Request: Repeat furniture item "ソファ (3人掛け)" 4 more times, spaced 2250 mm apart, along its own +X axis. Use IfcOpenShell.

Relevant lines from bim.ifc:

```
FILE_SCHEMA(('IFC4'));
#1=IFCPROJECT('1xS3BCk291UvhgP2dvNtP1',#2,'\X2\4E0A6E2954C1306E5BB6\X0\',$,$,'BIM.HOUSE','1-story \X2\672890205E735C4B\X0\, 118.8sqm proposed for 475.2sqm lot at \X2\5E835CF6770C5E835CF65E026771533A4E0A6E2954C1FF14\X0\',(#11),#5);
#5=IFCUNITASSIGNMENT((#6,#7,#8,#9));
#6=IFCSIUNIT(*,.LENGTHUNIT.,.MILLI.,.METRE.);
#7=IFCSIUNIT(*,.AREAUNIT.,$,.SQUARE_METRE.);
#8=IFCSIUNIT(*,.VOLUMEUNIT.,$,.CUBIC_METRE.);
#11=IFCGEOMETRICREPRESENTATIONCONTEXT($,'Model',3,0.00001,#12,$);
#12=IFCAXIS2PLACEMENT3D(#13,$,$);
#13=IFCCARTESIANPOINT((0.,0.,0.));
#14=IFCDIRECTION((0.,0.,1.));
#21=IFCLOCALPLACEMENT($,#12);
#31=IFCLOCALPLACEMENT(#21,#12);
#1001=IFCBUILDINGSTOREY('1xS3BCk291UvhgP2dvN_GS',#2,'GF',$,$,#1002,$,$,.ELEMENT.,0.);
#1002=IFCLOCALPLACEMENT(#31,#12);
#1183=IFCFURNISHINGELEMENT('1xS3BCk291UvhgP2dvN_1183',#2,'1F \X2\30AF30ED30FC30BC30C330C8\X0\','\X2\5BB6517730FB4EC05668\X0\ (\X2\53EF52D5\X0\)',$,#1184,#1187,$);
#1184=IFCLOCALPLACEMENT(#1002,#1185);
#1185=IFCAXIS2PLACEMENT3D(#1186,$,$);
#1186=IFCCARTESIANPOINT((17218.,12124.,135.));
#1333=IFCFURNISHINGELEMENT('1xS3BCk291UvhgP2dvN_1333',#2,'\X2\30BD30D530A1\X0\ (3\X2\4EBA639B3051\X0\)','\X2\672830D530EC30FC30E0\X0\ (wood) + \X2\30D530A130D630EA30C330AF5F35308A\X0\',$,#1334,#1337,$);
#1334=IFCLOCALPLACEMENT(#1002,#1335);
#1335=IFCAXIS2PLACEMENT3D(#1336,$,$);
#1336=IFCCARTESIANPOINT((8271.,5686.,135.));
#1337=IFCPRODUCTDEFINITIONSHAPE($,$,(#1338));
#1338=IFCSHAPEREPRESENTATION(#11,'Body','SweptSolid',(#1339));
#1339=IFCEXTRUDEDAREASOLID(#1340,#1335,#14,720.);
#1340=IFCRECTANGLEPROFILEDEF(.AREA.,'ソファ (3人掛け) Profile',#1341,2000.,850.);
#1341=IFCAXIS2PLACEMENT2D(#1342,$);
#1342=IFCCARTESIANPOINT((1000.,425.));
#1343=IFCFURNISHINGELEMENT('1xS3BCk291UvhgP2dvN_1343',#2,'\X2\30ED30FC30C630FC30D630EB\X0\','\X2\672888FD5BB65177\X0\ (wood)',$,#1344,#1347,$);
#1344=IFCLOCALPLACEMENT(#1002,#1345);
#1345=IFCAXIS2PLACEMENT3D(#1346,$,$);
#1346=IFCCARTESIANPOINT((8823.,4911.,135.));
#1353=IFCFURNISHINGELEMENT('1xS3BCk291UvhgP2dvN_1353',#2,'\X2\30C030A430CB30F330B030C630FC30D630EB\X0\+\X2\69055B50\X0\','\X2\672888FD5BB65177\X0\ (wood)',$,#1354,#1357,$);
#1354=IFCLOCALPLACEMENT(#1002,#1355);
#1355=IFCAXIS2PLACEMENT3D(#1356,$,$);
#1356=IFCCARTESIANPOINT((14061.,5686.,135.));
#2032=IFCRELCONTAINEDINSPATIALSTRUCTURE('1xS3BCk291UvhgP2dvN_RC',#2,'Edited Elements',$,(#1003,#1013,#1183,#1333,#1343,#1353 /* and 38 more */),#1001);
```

```python
import ifcopenshell
import ifcopenshell.api.geometry
import ifcopenshell.api.root
import ifcopenshell.util.element
import ifcopenshell.util.placement
import ifcopenshell.util.unit

model = ifcopenshell.open("bim.ifc")
unit_scale = ifcopenshell.util.unit.calculate_unit_scale(model)


def reuse_history(source, copy):
    """copy_class also copies each property set's owner history, people and application; keep the originals."""
    for rel in copy.IsDefinedBy:
        if rel.is_a("IfcRelDefinesByProperties") and (history := rel.RelatingPropertyDefinition.OwnerHistory):
            rel.RelatingPropertyDefinition.OwnerHistory = source.OwnerHistory
            ifcopenshell.util.element.remove_deep2(model, history)


source = model.by_id(1333)
base = ifcopenshell.util.placement.get_local_placement(source.ObjectPlacement)
step = base[:3, 0] * 2.25 / unit_scale

for i in range(1, 5):
    copy = ifcopenshell.api.root.copy_class(model, product=source)
    copy.Representation = ifcopenshell.util.element.copy_deep(
        model, source.Representation, exclude=["IfcGeometricRepresentationContext", "IfcRepresentationMap"]
    )
    reuse_history(source, copy)
    matrix = base.copy()
    matrix[:3, 3] += i * step
    print("added at", matrix[:3, 3].round(3) + 0.0)
    ifcopenshell.api.geometry.edit_object_placement(model, product=copy, matrix=matrix, is_si=False)

model.write("bim_rev.ifc")
```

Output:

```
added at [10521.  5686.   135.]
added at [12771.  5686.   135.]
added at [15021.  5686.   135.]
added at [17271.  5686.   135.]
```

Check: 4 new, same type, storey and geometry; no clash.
